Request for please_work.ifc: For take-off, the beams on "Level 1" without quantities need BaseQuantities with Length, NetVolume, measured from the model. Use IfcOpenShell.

First a look at what the model holds.

```python
import ifcopenshell
import ifcopenshell.util.element
import ifcopenshell.util.unit

model = ifcopenshell.open("please_work.ifc")
print(model.schema)
for unit_type in ("LENGTHUNIT", "AREAUNIT", "VOLUMEUNIT"):
    print(unit_type, ifcopenshell.util.unit.calculate_unit_scale(model, unit_type))
storey = next(s for s in model.by_type("IfcBuildingStorey") if s.Name == "Level 1")
beams = [e for e in ifcopenshell.util.element.get_decomposition(storey) if e.is_a("IfcBeam")]
for e in sorted(beams, key=lambda e: e.id()):
    print(e.id(), e.is_a(), e.Name, list(ifcopenshell.util.element.get_psets(e, qtos_only=True)), sep=" | ")
```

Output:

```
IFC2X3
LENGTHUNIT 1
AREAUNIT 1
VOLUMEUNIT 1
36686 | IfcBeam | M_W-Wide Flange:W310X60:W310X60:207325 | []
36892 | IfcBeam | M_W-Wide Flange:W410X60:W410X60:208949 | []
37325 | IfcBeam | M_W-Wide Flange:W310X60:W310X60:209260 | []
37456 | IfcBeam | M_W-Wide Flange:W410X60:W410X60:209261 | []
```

```python
import ifcopenshell
import ifcopenshell.api.pset
import ifcopenshell.geom
import ifcopenshell.util.element
import ifcopenshell.util.shape
import ifcopenshell.util.unit

model = ifcopenshell.open("please_work.ifc")
unit_scale = ifcopenshell.util.unit.calculate_unit_scale(model)
volume_scale = ifcopenshell.util.unit.calculate_unit_scale(model, "VOLUMEUNIT")
settings = ifcopenshell.geom.settings()

storey = next(s for s in model.by_type("IfcBuildingStorey") if s.Name == "Level 1")
beams = [e for e in ifcopenshell.util.element.get_decomposition(storey) if e.is_a("IfcBeam")]

for e in sorted(beams, key=lambda e: e.id()):
    if ifcopenshell.util.element.get_psets(e, qtos_only=True, should_inherit=False):
        continue
    # Geometry comes back in metres, in the element's own axes.
    shape = ifcopenshell.geom.create_shape(settings, e)
    values = {
        "Length": ifcopenshell.util.shape.get_max_xyz(shape.geometry) / unit_scale,
        "NetVolume": ifcopenshell.util.shape.get_volume(shape.geometry) / volume_scale,
    }
    qto = ifcopenshell.api.pset.add_qto(model, product=e, name="BaseQuantities")
    ifcopenshell.api.pset.edit_qto(model, qto=qto, properties=values)
    print(e.id(), {k: round(v, 3) for k, v in values.items()})

model.write("please_work_rev.ifc")
```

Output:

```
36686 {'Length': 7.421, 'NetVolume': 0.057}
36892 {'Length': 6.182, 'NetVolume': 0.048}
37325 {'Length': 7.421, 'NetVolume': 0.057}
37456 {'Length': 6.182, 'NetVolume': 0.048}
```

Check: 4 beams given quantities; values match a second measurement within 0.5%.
